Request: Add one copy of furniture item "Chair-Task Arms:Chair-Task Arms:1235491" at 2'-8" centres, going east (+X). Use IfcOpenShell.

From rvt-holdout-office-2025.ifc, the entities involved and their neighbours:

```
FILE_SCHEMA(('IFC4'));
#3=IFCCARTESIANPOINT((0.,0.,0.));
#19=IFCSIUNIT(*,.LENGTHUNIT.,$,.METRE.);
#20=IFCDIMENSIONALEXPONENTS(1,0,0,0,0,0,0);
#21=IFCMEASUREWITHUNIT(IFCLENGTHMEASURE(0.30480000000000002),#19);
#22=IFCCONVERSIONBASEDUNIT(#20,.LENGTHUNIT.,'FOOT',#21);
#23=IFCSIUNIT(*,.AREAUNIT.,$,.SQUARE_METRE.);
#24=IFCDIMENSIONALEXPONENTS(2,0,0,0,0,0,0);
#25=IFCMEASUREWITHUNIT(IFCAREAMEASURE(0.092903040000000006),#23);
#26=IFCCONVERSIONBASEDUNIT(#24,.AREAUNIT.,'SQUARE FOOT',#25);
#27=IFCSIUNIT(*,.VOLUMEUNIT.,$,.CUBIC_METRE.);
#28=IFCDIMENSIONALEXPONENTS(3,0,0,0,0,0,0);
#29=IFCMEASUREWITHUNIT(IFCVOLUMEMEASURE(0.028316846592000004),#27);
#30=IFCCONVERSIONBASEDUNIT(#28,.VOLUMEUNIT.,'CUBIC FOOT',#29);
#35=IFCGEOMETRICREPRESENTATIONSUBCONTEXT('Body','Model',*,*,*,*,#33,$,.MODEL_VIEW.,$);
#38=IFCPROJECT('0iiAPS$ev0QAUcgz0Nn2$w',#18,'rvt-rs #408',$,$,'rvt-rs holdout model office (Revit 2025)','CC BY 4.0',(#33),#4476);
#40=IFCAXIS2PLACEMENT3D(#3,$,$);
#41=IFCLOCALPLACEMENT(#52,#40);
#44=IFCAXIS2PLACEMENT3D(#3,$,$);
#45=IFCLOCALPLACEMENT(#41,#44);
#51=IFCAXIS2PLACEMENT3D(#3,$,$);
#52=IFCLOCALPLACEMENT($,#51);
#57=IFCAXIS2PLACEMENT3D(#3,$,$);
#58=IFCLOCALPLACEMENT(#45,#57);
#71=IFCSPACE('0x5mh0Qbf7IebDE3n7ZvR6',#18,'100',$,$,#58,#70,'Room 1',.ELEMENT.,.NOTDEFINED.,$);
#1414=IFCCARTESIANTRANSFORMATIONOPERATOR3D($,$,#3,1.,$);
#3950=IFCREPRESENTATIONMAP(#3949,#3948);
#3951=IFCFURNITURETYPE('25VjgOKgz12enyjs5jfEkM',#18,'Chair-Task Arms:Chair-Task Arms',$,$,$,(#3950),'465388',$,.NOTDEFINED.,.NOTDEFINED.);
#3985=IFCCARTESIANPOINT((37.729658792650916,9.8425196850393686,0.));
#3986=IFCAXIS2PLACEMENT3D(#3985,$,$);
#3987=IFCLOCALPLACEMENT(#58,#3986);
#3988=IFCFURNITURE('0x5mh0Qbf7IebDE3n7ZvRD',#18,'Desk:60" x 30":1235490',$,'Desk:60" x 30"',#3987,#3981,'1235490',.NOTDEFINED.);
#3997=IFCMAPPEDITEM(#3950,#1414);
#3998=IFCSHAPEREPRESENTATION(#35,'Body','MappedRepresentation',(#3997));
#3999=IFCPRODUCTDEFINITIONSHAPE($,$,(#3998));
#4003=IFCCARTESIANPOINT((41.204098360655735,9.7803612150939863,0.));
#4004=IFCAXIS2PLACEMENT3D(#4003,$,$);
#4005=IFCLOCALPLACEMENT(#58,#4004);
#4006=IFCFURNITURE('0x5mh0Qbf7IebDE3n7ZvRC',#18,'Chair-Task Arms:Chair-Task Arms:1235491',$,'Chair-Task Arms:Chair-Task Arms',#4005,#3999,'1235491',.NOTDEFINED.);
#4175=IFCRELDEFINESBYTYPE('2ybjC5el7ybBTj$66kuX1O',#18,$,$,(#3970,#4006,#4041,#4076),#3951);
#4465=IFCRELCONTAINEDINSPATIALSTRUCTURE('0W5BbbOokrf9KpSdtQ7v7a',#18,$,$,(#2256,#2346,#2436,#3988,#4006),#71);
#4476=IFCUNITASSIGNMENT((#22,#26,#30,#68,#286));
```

```python
import numpy as np
import ifcopenshell
import ifcopenshell.api.geometry
import ifcopenshell.api.root
import ifcopenshell.util.element
import ifcopenshell.util.placement
import ifcopenshell.util.unit

model = ifcopenshell.open("rvt-holdout-office-2025.ifc")
unit_scale = ifcopenshell.util.unit.calculate_unit_scale(model)


def reuse_history(source, copy):
    """copy_class also copies each property set's owner history, people and application; keep the originals."""
    for rel in copy.IsDefinedBy:
        if rel.is_a("IfcRelDefinesByProperties") and (history := rel.RelatingPropertyDefinition.OwnerHistory):
            rel.RelatingPropertyDefinition.OwnerHistory = source.OwnerHistory
            ifcopenshell.util.element.remove_deep2(model, history)


source = model.by_guid("0x5mh0Qbf7IebDE3n7ZvRC")
base = ifcopenshell.util.placement.get_local_placement(source.ObjectPlacement)
step = np.array([1.0, 0.0, 0.0]) * 32 * 0.0254 / unit_scale

for i in range(1, 2):
    copy = ifcopenshell.api.root.copy_class(model, product=source)
    copy.Representation = ifcopenshell.util.element.copy_deep(
        model, source.Representation, exclude=["IfcGeometricRepresentationContext", "IfcRepresentationMap"]
    )
    copy.Name = "Chair-Task Arms:Chair-Task Arms"
    copy.Tag = None
    reuse_history(source, copy)
    matrix = base.copy()
    matrix[:3, 3] += i * step
    print("added at", matrix[:3, 3].round(3) + 0.0)
    ifcopenshell.api.geometry.edit_object_placement(model, product=copy, matrix=matrix, is_si=False)

model.write("rvt-holdout-office-2025_v2.ifc")
```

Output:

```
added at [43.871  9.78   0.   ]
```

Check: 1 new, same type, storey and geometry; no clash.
